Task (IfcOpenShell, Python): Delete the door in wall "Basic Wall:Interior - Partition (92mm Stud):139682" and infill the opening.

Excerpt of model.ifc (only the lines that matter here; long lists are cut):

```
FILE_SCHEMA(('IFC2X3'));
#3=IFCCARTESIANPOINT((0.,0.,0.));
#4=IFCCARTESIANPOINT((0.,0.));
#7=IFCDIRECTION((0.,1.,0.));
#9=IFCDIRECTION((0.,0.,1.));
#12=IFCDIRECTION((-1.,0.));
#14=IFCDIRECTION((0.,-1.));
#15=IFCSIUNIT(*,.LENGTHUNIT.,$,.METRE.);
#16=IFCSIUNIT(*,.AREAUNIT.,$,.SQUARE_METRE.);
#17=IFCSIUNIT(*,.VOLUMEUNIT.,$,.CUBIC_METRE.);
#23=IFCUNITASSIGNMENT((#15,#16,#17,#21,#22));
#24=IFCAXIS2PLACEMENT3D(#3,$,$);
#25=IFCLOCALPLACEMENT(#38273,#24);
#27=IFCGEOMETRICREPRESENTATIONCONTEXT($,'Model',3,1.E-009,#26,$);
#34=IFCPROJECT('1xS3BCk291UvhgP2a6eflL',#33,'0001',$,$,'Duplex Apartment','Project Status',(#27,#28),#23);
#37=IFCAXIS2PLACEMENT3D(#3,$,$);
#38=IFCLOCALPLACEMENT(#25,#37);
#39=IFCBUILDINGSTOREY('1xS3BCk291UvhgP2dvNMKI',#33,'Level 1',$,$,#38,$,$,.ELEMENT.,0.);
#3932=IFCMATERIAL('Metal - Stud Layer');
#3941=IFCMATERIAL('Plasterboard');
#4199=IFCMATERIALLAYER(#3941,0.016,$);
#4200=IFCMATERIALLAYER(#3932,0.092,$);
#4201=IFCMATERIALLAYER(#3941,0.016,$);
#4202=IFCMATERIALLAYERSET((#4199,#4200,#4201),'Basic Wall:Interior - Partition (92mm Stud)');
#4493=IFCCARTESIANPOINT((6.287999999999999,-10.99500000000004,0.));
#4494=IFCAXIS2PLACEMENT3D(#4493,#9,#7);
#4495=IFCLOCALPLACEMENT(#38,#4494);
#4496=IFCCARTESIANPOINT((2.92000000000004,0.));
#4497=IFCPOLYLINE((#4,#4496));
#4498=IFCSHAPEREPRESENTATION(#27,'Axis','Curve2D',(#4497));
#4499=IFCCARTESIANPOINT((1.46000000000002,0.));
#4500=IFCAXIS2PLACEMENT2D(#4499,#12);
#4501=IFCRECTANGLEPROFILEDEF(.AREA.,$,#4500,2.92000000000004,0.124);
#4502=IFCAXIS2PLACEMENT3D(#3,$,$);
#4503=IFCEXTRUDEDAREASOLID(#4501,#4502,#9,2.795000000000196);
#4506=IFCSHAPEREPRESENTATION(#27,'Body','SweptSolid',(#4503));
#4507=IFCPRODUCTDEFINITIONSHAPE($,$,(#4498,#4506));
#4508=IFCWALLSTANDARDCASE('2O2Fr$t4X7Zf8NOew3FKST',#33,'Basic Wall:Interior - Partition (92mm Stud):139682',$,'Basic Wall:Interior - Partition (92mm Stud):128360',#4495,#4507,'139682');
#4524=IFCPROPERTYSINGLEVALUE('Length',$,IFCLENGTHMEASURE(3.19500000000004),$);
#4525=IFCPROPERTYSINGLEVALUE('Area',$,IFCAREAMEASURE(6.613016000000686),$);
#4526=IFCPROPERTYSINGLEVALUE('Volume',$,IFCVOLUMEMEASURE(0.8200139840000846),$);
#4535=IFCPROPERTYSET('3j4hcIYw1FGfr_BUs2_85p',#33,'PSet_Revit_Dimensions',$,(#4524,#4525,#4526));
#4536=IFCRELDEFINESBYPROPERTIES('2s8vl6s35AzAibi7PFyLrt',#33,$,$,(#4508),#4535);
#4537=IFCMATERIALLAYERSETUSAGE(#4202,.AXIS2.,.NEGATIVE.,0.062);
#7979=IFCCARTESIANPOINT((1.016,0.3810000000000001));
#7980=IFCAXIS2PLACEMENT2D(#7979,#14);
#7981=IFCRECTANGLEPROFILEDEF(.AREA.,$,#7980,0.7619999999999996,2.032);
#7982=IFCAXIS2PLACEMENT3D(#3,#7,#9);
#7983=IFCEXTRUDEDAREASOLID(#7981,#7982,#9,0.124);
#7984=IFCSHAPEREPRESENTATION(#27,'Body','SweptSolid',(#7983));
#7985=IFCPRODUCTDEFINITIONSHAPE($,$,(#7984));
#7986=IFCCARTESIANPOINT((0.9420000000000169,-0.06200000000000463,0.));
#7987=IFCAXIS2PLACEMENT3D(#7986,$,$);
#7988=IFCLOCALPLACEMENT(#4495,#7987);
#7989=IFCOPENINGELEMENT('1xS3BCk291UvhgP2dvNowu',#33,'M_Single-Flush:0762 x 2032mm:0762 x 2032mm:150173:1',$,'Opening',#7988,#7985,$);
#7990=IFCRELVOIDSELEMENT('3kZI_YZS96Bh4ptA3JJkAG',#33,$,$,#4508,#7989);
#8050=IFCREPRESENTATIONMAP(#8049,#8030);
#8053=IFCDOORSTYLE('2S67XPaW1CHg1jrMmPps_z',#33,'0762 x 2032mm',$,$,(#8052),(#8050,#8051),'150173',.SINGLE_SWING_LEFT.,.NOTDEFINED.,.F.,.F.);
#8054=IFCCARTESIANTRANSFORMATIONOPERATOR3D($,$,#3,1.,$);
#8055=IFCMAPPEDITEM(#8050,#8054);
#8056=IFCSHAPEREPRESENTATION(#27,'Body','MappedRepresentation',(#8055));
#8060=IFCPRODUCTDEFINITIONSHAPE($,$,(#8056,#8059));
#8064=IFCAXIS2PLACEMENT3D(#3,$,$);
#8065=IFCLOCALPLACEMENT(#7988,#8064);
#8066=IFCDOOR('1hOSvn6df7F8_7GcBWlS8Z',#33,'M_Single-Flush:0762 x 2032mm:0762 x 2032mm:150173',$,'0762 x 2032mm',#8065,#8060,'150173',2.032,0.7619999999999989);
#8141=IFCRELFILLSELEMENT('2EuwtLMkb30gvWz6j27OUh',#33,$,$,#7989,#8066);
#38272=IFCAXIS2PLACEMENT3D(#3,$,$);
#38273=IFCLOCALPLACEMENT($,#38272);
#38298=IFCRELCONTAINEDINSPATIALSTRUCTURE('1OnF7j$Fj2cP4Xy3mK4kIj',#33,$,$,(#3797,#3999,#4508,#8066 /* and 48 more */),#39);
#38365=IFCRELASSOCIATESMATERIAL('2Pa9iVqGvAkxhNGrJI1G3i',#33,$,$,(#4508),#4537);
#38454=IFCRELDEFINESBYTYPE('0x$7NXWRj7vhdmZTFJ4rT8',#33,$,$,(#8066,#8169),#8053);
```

```python
import ifcopenshell
import ifcopenshell.api.feature
import ifcopenshell.api.pset
import ifcopenshell.api.root
import ifcopenshell.geom
import ifcopenshell.util.element
import ifcopenshell.util.shape
import ifcopenshell.util.unit

model = ifcopenshell.open("model.ifc")
area_scale = ifcopenshell.util.unit.calculate_unit_scale(model, "AREAUNIT")
volume_scale = ifcopenshell.util.unit.calculate_unit_scale(model, "VOLUMEUNIT")
settings = ifcopenshell.geom.settings()


def volume(element):
    """Net volume in cubic metres, openings subtracted."""
    shape = ifcopenshell.geom.create_shape(settings, element)
    return ifcopenshell.util.shape.get_volume(shape.geometry)


door = model.by_guid("1hOSvn6df7F8_7GcBWlS8Z")
opening = door.FillsVoids[0].RelatingOpeningElement
wall = opening.VoidsElements[0].RelatingBuildingElement
before = volume(wall)

ifcopenshell.api.root.remove_product(model, product=door)
ifcopenshell.api.feature.remove_feature(model, feature=opening)

after = volume(wall)
thickness = 0.124  # wall thickness in metres

# Update the wall's stored quantities.
pset = model.by_id(ifcopenshell.util.element.get_pset(wall, "PSet_Revit_Dimensions", should_inherit=False)["id"])
ifcopenshell.api.pset.edit_pset(model, pset=pset, properties={
    "Area": model.create_entity("IfcAreaMeasure", after / thickness / area_scale),
    "Volume": model.create_entity("IfcVolumeMeasure", after / volume_scale),
})

print(f"wall volume {before:.3f} -> {after:.3f} m3")

model.write("model_edited.ifc")
```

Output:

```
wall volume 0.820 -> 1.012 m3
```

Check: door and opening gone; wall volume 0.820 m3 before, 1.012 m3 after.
